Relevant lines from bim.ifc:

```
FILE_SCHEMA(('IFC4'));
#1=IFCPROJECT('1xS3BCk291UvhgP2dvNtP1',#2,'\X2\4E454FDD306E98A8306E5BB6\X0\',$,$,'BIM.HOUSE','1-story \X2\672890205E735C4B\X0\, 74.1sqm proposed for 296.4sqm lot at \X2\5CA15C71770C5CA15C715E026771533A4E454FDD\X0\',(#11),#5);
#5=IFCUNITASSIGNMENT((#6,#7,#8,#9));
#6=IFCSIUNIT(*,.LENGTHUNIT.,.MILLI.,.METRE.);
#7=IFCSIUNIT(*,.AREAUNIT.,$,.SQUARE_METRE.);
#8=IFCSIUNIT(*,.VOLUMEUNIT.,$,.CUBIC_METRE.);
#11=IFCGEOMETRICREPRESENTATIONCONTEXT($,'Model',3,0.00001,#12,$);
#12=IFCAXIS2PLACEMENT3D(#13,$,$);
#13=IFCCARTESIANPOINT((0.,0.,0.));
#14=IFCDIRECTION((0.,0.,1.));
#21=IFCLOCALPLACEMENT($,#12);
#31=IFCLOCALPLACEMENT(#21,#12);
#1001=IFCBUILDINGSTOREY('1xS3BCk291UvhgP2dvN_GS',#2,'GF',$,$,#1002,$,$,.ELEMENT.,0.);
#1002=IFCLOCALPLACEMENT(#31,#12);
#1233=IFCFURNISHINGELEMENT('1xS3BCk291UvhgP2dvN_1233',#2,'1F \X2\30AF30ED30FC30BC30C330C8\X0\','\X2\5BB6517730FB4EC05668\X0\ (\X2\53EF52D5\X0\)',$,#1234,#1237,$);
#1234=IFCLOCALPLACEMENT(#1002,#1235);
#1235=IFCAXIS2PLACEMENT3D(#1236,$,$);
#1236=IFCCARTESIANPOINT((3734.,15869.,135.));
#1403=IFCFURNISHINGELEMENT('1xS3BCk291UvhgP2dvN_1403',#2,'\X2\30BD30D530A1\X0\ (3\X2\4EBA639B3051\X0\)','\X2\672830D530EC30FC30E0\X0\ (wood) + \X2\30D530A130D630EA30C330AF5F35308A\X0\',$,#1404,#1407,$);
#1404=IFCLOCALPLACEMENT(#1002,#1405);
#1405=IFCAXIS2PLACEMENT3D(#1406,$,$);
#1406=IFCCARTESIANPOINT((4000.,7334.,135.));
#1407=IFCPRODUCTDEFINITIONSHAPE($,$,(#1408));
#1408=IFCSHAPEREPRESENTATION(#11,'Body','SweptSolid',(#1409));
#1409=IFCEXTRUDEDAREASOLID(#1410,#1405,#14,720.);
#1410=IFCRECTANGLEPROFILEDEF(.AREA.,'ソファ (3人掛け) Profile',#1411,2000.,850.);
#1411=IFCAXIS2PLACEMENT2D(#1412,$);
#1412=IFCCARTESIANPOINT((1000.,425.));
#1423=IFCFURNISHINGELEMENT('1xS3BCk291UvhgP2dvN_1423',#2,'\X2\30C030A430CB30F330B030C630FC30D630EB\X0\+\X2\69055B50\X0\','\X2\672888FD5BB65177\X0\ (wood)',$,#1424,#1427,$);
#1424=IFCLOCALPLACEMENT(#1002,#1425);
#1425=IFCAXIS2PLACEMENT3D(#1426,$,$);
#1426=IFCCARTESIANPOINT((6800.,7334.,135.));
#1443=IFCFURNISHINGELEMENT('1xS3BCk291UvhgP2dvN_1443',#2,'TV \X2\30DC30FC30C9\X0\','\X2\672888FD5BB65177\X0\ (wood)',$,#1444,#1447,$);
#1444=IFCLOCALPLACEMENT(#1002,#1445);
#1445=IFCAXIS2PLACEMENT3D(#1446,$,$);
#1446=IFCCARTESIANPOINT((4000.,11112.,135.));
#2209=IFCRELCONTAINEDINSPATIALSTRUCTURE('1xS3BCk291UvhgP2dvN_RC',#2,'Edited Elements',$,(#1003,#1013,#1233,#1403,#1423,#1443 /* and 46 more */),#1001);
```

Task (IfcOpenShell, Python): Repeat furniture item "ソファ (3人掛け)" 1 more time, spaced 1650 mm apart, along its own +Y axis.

```python
import ifcopenshell
import ifcopenshell.api.geometry
import ifcopenshell.api.root
import ifcopenshell.util.element
import ifcopenshell.util.placement
import ifcopenshell.util.unit

model = ifcopenshell.open("bim.ifc")
unit_scale = ifcopenshell.util.unit.calculate_unit_scale(model)


def reuse_history(source, copy):
    """copy_class also copies each property set's owner history, people and application; keep the originals."""
    for rel in copy.IsDefinedBy:
        if rel.is_a("IfcRelDefinesByProperties") and (history := rel.RelatingPropertyDefinition.OwnerHistory):
            rel.RelatingPropertyDefinition.OwnerHistory = source.OwnerHistory
            ifcopenshell.util.element.remove_deep2(model, history)


source = model.by_guid("1xS3BCk291UvhgP2dvN_1403")
base = ifcopenshell.util.placement.get_local_placement(source.ObjectPlacement)
step = base[:3, 1] * 1.65 / unit_scale

for i in range(1, 2):
    copy = ifcopenshell.api.root.copy_class(model, product=source)
    copy.Representation = ifcopenshell.util.element.copy_deep(
        model, source.Representation, exclude=["IfcGeometricRepresentationContext", "IfcRepresentationMap"]
    )
    reuse_history(source, copy)
    matrix = base.copy()
    matrix[:3, 3] += i * step
    print("added at", matrix[:3, 3].round(3) + 0.0)
    ifcopenshell.api.geometry.edit_object_placement(model, product=copy, matrix=matrix, is_si=False)

model.write("bim_rev.ifc")
```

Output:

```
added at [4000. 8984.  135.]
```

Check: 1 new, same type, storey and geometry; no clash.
